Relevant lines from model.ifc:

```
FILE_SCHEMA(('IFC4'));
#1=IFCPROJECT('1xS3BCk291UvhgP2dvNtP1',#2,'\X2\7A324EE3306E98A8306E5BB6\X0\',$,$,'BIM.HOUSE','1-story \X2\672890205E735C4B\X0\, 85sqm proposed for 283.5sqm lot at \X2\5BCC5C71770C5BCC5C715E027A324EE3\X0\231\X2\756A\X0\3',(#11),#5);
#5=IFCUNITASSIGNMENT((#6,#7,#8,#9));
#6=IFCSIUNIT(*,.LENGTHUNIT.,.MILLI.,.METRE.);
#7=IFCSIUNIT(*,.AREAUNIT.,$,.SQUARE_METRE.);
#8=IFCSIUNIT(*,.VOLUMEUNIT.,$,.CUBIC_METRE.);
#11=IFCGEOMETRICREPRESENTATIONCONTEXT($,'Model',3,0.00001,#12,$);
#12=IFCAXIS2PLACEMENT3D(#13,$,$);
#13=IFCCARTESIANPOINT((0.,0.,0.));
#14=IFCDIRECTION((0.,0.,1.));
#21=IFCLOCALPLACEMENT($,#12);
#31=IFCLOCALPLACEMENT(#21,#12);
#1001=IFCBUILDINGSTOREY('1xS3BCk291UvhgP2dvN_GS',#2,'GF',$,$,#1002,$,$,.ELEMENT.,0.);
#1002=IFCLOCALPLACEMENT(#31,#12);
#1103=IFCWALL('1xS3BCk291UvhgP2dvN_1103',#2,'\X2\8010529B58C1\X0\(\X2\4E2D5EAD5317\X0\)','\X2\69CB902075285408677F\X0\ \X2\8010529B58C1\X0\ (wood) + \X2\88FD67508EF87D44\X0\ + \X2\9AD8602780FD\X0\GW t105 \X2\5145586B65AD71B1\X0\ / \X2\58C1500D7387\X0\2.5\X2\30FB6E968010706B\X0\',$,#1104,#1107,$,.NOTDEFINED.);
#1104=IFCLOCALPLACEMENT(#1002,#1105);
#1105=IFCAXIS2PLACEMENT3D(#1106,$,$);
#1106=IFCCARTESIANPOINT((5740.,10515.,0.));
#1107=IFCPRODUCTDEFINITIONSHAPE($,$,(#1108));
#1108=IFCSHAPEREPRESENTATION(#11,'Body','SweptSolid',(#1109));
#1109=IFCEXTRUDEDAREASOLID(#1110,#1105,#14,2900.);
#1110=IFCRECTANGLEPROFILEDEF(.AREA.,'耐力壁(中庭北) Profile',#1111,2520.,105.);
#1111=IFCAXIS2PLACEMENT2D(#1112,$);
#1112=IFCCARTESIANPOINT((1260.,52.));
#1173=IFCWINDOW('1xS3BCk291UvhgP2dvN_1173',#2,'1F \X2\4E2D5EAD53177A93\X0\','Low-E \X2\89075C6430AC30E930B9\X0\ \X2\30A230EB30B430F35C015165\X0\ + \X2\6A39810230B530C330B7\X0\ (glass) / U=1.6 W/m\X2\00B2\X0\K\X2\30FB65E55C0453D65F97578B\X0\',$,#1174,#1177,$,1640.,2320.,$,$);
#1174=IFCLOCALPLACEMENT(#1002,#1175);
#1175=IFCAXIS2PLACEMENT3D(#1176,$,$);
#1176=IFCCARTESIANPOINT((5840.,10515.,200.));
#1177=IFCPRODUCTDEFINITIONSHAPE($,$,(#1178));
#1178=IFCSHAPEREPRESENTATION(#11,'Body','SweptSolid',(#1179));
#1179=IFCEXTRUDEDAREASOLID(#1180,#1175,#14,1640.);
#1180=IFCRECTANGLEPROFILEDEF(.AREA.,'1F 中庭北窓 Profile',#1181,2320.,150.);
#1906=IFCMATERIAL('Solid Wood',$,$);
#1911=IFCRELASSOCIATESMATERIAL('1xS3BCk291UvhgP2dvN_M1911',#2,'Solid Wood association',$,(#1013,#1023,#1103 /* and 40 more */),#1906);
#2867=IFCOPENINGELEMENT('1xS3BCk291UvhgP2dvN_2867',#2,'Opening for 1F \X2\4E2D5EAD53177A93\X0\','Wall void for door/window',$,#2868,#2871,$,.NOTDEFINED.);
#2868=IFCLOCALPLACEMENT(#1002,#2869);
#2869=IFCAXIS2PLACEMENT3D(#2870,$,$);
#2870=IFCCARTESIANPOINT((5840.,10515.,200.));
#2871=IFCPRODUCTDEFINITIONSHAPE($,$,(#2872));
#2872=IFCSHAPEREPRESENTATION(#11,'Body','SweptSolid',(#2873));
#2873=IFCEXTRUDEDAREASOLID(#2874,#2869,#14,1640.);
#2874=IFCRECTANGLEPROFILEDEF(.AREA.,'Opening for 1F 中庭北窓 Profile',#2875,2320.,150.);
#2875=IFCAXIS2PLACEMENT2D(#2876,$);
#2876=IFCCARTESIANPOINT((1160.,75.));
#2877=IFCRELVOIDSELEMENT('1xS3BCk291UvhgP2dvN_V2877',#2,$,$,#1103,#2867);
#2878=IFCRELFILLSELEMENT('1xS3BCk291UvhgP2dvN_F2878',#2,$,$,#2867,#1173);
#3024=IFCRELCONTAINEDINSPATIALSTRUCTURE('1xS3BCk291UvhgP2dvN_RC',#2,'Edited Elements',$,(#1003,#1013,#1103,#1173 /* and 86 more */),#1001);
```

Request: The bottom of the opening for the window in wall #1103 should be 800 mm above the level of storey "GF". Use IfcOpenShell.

```python
import numpy as np
import ifcopenshell
import ifcopenshell.api.geometry
import ifcopenshell.geom
import ifcopenshell.util.element
import ifcopenshell.util.placement
import ifcopenshell.util.shape
import ifcopenshell.util.unit

model = ifcopenshell.open("model.ifc")
unit_scale = ifcopenshell.util.unit.calculate_unit_scale(model)

window = model.by_id(1173)
opening = window.FillsVoids[0].RelatingOpeningElement
storey = ifcopenshell.util.element.get_container(window, ifc_class="IfcBuildingStorey")
level = ifcopenshell.util.placement.get_local_placement(storey.ObjectPlacement)[2, 3]

# The opening's origin need not be at the sill, so measure its lowest point.
shape = ifcopenshell.geom.create_shape(ifcopenshell.geom.settings(), opening)
bottom = ifcopenshell.util.shape.get_shape_bottom_elevation(shape, shape.geometry) / unit_scale
dz = level + 800.0 - bottom

shift = np.array([0.0, 0.0, dz])
# The window is not placed relative to its opening, so move both.
for product in (opening, window):
    matrix = ifcopenshell.util.placement.get_local_placement(product.ObjectPlacement)
    matrix[:3, 3] += shift
    ifcopenshell.api.geometry.edit_object_placement(model, product=product, matrix=matrix, is_si=False)

print(f"moved by {dz * unit_scale:+.3f} m")

model.write("model-out.ifc")
```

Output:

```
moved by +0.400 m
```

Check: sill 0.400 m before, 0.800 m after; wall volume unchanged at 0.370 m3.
